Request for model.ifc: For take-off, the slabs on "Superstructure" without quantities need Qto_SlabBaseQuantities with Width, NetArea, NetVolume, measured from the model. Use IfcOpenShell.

First a look at what the model holds.

```python
import ifcopenshell
import ifcopenshell.util.element
import ifcopenshell.util.unit

model = ifcopenshell.open("model.ifc")
print(model.schema)
for unit_type in ("LENGTHUNIT", "AREAUNIT", "VOLUMEUNIT"):
    print(unit_type, ifcopenshell.util.unit.calculate_unit_scale(model, unit_type))
storey = next(s for s in model.by_type("IfcBuildingStorey") if s.Name == "Superstructure")
slabs = [e for e in ifcopenshell.util.element.get_decomposition(storey) if e.is_a("IfcSlab")]
for e in sorted(slabs, key=lambda e: e.id()):
    print(e.id(), e.is_a(), e.Name, list(ifcopenshell.util.element.get_psets(e, qtos_only=True)), sep=" | ")
```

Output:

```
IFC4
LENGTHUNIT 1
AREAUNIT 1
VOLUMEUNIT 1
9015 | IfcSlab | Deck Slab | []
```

```python
import ifcopenshell
import ifcopenshell.api.pset
import ifcopenshell.geom
import ifcopenshell.util.element
import ifcopenshell.util.shape
import ifcopenshell.util.unit

model = ifcopenshell.open("model.ifc")
unit_scale = ifcopenshell.util.unit.calculate_unit_scale(model)
area_scale = ifcopenshell.util.unit.calculate_unit_scale(model, "AREAUNIT")
volume_scale = ifcopenshell.util.unit.calculate_unit_scale(model, "VOLUMEUNIT")
settings = ifcopenshell.geom.settings()

storey = next(s for s in model.by_type("IfcBuildingStorey") if s.Name == "Superstructure")
slabs = [e for e in ifcopenshell.util.element.get_decomposition(storey) if e.is_a("IfcSlab")]

for e in sorted(slabs, key=lambda e: e.id()):
    if ifcopenshell.util.element.get_psets(e, qtos_only=True, should_inherit=False):
        continue
    # Geometry comes back in metres, in the element's own axes.
    shape = ifcopenshell.geom.create_shape(settings, e)
    values = {
        "Width": ifcopenshell.util.shape.get_z(shape.geometry) / unit_scale,
        "NetArea": ifcopenshell.util.shape.get_footprint_area(shape.geometry) / area_scale,
        "NetVolume": ifcopenshell.util.shape.get_volume(shape.geometry) / volume_scale,
    }
    qto = ifcopenshell.api.pset.add_qto(model, product=e, name="Qto_SlabBaseQuantities")
    ifcopenshell.api.pset.edit_qto(model, qto=qto, properties=values)
    print(e.id(), {k: round(v, 3) for k, v in values.items()})

model.write("model_updated.ifc")
```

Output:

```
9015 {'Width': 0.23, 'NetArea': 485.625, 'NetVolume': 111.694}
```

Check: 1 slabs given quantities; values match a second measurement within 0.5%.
